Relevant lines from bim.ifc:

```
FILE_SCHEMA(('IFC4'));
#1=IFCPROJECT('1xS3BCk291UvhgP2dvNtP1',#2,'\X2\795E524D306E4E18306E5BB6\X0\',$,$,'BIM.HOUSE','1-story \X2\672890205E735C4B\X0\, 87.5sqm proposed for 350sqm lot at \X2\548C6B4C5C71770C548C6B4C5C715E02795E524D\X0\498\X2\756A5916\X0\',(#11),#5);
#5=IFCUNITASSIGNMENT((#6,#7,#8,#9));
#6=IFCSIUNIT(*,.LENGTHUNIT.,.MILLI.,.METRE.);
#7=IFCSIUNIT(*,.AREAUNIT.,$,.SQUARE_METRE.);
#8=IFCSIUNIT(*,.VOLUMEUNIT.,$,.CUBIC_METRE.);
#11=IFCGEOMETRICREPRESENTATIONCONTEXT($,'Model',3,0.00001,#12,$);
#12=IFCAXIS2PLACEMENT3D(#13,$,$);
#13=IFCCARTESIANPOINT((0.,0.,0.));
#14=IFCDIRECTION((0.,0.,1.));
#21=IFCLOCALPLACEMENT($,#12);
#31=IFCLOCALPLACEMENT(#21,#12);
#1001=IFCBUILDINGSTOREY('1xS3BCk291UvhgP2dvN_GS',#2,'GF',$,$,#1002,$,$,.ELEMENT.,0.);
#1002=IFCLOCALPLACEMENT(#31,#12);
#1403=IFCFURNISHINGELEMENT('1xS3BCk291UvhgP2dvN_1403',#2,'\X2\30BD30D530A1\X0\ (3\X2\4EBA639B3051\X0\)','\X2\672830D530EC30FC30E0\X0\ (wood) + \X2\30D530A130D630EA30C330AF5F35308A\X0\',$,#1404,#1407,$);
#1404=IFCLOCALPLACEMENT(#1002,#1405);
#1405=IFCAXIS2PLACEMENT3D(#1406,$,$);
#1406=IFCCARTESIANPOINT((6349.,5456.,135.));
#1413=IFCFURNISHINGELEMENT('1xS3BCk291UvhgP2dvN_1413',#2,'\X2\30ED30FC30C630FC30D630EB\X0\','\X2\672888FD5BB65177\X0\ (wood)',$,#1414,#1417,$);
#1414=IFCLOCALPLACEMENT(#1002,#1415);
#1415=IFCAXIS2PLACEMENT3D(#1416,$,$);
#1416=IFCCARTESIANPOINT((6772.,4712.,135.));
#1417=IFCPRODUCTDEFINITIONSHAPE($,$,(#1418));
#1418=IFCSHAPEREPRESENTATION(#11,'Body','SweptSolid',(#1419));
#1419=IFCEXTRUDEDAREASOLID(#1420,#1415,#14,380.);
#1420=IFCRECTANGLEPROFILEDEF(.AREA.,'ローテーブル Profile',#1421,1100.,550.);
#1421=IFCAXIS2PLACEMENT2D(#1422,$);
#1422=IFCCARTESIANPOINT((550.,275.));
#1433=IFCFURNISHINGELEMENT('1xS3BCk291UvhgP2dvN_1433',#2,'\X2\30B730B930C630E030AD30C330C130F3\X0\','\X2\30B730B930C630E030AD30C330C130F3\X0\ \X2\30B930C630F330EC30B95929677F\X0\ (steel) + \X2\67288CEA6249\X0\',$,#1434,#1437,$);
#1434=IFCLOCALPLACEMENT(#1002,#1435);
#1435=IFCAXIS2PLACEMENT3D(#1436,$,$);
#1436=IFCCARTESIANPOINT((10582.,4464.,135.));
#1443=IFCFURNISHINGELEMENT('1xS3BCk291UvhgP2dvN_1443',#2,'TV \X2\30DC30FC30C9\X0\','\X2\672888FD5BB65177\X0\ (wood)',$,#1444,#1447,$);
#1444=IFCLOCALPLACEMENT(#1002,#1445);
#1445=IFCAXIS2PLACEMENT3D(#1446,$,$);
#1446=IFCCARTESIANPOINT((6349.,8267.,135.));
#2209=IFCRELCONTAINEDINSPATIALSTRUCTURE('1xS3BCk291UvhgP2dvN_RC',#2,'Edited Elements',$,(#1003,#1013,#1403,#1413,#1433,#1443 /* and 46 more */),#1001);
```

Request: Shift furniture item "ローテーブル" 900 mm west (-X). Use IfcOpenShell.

```python
import ifcopenshell
import ifcopenshell.api.geometry
import ifcopenshell.util.placement
import ifcopenshell.util.unit

model = ifcopenshell.open("bim.ifc")
unit_scale = ifcopenshell.util.unit.calculate_unit_scale(model)

item = model.by_guid("1xS3BCk291UvhgP2dvN_1413")
matrix = ifcopenshell.util.placement.get_local_placement(item.ObjectPlacement)
matrix[0, 3] -= 0.9 / unit_scale
ifcopenshell.api.geometry.edit_object_placement(model, product=item, matrix=matrix, is_si=False)

print(ifcopenshell.util.placement.get_local_placement(item.ObjectPlacement).round(3) + 0.0)

model.write("bim_v2.ifc")
```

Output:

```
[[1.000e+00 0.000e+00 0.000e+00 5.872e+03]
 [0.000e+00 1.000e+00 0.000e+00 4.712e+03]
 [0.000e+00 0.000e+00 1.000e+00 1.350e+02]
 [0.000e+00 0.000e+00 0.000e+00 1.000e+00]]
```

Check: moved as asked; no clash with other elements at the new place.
